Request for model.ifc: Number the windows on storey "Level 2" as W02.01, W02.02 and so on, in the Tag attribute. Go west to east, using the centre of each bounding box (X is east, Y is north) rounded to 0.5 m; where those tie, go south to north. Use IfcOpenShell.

First a look at what the model holds.

```python
import ifcopenshell
import ifcopenshell.util.element
import ifcopenshell.util.placement

model = ifcopenshell.open("model.ifc")
print(model.schema)
storey = next(s for s in model.by_type("IfcBuildingStorey") if s.Name == "Level 2")
windows = [e for e in ifcopenshell.util.element.get_decomposition(storey) if e.is_a("IfcWindow")]
for e in sorted(windows, key=lambda e: e.id()):
    origin = ifcopenshell.util.placement.get_local_placement(e.ObjectPlacement)[:3, 3]
    print(e.id(), e.Tag, e.Name, origin.round(2) + 0.0, sep=" | ")
```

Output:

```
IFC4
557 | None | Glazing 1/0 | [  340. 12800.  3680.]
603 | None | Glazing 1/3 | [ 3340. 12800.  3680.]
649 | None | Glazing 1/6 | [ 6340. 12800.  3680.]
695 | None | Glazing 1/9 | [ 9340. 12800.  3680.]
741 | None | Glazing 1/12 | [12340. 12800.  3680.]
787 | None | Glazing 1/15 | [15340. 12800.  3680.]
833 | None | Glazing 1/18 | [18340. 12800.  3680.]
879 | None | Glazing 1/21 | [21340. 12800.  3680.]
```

```python
import ifcopenshell
import ifcopenshell.geom
import ifcopenshell.util.element
import ifcopenshell.util.shape

model = ifcopenshell.open("model.ifc")
settings = ifcopenshell.geom.settings()
settings.set("use-world-coords", True)


def centre(element):
    shape = ifcopenshell.geom.create_shape(settings, element)
    return ifcopenshell.util.shape.get_bbox_centroid(shape.geometry)


storey = next(s for s in model.by_type("IfcBuildingStorey") if s.Name == "Level 2")
windows = [e for e in ifcopenshell.util.element.get_decomposition(storey) if e.is_a("IfcWindow")]

# Insertion points can sit at a corner or the storey origin, so sort by the geometry (in metres).
centres = {e: centre(e) for e in windows}
windows.sort(key=lambda e: (round(centres[e][0] / 0.5), centres[e][1]))

for i, e in enumerate(windows, start=1):
    number = f"W02.{i:02d}"
    e.Tag = number
    print(e.id(), number)

model.write("model-out.ifc")
```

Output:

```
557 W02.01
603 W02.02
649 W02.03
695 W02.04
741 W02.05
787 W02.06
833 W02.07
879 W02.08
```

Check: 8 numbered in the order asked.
